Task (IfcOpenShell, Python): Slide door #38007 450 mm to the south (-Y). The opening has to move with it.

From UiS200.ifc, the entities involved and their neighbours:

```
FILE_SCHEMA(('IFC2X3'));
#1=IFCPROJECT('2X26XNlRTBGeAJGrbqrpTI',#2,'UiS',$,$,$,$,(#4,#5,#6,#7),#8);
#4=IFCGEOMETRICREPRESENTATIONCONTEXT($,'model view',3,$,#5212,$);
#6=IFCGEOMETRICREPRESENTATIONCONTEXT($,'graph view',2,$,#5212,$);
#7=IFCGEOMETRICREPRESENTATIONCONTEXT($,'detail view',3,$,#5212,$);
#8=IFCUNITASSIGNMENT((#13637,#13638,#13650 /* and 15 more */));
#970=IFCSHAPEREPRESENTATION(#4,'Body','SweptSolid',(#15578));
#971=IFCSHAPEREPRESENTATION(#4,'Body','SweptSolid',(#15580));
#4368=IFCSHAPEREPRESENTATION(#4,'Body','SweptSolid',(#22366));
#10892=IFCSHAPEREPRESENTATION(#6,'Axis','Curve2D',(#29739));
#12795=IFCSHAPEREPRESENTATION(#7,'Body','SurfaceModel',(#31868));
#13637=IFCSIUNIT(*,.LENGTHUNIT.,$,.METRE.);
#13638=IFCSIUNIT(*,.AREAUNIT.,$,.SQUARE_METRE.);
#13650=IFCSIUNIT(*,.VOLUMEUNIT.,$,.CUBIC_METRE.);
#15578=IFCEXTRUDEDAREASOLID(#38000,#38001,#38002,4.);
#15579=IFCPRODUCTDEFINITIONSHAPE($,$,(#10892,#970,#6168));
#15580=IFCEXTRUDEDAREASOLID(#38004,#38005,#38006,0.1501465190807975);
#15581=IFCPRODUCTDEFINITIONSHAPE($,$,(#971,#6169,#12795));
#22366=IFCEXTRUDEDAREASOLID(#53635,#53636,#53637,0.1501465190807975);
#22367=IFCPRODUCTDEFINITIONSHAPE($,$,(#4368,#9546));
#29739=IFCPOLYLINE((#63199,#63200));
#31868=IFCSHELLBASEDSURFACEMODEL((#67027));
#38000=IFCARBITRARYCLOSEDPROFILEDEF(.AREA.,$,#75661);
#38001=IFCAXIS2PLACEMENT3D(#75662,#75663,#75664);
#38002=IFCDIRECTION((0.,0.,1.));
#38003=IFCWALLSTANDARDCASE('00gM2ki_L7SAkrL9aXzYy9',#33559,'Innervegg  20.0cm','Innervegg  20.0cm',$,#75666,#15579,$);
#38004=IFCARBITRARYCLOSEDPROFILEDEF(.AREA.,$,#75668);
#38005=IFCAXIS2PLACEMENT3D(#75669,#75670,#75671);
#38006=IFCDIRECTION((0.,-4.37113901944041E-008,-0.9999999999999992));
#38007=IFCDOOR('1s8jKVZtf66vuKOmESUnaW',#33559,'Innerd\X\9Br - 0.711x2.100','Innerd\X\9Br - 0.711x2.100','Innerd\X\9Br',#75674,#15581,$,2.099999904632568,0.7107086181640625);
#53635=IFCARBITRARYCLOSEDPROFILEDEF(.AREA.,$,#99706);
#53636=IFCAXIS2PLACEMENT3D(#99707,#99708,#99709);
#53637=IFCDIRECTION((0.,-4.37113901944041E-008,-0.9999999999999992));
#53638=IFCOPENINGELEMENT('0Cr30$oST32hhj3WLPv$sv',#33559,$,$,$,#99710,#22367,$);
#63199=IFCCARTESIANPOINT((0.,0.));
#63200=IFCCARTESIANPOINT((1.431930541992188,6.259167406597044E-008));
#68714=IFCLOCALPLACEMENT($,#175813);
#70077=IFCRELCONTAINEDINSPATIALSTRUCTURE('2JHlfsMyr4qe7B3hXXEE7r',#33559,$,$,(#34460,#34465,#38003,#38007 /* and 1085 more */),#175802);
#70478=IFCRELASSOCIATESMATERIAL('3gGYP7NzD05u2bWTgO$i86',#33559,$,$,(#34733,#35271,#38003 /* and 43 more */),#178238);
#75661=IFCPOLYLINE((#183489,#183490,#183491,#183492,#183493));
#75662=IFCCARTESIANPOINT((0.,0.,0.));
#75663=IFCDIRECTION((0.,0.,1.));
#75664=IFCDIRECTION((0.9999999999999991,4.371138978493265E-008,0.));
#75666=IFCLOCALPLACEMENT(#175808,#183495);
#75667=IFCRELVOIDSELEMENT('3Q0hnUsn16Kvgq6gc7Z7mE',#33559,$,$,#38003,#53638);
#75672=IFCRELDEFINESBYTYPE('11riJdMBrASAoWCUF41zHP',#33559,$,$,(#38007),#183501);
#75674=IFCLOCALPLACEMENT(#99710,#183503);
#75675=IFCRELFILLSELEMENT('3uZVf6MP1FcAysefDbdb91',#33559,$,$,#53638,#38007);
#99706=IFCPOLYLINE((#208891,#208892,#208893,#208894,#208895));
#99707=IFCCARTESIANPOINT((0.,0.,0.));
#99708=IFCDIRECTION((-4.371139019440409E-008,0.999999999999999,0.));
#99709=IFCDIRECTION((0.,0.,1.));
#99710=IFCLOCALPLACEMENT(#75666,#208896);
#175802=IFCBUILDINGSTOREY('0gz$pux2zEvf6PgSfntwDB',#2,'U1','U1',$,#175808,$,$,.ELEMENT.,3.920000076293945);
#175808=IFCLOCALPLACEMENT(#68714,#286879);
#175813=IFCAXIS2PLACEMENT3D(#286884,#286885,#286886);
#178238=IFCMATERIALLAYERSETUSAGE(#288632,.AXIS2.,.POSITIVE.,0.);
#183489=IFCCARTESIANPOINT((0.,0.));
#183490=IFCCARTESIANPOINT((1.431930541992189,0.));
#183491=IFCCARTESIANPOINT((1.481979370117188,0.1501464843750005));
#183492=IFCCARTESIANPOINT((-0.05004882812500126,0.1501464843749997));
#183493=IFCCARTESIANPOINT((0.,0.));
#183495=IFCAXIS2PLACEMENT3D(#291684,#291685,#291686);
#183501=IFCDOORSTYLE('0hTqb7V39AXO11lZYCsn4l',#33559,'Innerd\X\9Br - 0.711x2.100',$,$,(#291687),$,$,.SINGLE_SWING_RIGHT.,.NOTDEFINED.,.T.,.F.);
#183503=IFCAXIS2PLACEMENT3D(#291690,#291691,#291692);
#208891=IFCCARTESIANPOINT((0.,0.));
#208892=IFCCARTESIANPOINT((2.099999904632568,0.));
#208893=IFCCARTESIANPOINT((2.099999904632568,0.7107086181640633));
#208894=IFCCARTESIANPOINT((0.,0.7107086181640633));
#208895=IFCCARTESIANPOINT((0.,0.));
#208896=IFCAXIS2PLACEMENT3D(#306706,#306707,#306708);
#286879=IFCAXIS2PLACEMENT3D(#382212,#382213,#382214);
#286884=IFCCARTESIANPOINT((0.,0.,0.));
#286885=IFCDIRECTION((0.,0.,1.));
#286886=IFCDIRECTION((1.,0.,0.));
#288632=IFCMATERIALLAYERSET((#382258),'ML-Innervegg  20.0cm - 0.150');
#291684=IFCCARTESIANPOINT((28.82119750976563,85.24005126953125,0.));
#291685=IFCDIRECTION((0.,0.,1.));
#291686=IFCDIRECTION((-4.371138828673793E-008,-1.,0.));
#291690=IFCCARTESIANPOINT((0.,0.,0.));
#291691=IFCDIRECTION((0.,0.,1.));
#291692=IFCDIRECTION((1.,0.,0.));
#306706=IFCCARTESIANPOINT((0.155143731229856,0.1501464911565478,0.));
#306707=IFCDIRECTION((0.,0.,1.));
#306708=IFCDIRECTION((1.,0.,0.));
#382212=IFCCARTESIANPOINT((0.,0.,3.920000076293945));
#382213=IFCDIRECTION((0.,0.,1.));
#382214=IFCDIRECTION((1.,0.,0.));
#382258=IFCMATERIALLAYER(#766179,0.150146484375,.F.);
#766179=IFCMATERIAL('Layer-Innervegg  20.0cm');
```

```python
import ifcopenshell
import ifcopenshell.api.geometry
import ifcopenshell.util.placement

model = ifcopenshell.open("UiS200.ifc")

door = model.by_id(38007)
opening = door.FillsVoids[0].RelatingOpeningElement
wall = opening.VoidsElements[0].RelatingBuildingElement

wall_matrix = ifcopenshell.util.placement.get_local_placement(wall.ObjectPlacement)
shift = wall_matrix[:3, 0] * 0.45
before = ifcopenshell.util.placement.get_local_placement(door.ObjectPlacement)[:3, 3].copy()

# The door is placed relative to its opening, so it follows when the opening moves.
matrix = ifcopenshell.util.placement.get_local_placement(opening.ObjectPlacement)
matrix[:3, 3] += shift
ifcopenshell.api.geometry.edit_object_placement(
    model, product=opening, matrix=matrix, is_si=False, should_transform_children=True
)

after = ifcopenshell.util.placement.get_local_placement(door.ObjectPlacement)[:3, 3]
print("door moved by", (after - before).round(3) + 0.0)

model.write("UiS200-out.ifc")
```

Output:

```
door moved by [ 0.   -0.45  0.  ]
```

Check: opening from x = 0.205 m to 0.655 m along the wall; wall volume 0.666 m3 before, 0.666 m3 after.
